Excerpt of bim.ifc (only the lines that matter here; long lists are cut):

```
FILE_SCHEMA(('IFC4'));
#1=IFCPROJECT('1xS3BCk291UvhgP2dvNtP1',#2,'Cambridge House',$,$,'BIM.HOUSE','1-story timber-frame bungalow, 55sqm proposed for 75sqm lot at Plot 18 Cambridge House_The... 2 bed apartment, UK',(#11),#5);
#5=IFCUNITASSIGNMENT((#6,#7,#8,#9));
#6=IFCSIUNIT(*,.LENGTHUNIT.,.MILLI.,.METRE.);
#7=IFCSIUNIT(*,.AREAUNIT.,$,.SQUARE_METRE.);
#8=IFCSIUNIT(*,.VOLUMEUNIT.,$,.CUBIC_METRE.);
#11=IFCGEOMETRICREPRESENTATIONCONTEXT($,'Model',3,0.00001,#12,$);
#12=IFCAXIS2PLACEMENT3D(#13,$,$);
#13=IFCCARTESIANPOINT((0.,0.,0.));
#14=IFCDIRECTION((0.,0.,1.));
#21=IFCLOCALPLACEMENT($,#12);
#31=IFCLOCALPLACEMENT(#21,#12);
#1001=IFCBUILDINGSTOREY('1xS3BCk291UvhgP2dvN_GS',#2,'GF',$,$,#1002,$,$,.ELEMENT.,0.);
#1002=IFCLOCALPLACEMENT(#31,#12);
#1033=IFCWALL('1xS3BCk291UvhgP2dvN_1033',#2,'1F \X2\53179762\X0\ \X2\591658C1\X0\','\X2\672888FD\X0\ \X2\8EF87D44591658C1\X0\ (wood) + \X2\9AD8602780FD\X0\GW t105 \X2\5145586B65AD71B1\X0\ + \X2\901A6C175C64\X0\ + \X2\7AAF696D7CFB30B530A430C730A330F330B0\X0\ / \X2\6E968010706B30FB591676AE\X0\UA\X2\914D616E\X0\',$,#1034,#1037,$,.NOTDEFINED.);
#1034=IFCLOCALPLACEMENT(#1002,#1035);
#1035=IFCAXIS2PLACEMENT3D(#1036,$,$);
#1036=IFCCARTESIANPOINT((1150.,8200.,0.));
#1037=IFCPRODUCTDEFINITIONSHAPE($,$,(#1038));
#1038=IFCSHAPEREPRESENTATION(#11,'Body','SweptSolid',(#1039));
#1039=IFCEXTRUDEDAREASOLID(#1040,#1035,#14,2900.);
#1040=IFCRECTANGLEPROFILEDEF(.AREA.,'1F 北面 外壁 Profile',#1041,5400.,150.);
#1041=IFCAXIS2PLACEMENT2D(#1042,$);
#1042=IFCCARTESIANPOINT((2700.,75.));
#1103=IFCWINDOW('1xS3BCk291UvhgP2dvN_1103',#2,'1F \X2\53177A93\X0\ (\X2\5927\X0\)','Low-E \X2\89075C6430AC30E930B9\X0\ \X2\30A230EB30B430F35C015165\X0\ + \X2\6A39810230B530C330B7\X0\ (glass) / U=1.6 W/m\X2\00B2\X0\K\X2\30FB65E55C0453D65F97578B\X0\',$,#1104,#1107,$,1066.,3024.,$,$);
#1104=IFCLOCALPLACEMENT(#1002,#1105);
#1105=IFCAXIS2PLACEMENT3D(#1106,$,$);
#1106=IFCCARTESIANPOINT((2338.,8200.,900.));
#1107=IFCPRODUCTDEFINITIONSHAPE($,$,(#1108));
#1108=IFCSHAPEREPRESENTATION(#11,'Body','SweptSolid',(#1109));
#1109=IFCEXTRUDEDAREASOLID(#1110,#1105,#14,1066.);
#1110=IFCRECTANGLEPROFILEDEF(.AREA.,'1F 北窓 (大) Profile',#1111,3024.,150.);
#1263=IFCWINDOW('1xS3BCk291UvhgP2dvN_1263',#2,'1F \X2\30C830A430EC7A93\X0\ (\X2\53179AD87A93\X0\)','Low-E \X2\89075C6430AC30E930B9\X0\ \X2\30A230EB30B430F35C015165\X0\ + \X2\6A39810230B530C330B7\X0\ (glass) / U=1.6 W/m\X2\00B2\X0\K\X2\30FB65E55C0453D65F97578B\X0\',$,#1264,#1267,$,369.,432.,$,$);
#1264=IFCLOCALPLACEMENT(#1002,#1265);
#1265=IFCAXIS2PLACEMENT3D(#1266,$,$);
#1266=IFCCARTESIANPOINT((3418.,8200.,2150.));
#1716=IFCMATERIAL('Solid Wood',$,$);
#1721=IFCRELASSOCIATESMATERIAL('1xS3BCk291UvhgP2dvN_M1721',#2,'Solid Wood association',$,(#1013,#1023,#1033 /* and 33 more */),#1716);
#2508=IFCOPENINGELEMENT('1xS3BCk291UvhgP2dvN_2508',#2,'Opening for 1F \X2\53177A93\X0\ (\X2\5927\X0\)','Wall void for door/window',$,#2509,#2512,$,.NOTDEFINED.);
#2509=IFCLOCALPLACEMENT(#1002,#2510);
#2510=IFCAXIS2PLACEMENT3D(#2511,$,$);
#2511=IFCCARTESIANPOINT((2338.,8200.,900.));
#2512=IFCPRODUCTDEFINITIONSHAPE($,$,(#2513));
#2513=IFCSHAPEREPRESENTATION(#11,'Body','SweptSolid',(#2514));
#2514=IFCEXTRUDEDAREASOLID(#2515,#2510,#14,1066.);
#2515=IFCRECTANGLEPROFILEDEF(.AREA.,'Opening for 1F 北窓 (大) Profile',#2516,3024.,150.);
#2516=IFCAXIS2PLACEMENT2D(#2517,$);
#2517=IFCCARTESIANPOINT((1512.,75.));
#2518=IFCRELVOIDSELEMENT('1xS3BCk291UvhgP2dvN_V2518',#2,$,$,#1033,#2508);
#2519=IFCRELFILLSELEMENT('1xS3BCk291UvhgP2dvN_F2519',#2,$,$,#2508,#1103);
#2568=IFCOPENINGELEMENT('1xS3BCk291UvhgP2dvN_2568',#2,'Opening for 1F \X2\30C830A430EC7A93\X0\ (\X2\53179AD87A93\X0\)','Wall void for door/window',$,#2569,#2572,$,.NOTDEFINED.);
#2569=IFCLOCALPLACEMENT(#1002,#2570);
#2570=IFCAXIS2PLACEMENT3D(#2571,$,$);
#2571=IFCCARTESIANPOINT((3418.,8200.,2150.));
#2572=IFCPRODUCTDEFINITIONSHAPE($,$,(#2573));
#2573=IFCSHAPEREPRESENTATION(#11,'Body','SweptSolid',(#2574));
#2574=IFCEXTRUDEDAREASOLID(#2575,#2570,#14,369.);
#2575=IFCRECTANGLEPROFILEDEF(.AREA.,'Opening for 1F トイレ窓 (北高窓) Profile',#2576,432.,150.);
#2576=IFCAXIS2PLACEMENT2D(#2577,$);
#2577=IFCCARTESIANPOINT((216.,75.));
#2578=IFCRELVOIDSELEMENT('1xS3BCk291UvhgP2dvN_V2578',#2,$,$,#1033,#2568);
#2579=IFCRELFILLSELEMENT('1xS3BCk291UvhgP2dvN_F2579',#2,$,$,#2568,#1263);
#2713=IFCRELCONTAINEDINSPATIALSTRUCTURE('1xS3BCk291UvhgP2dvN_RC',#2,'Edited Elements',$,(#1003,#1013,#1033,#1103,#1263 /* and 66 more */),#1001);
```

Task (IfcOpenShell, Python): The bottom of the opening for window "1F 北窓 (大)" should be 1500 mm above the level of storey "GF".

```python
import numpy as np
import ifcopenshell
import ifcopenshell.api.geometry
import ifcopenshell.geom
import ifcopenshell.util.element
import ifcopenshell.util.placement
import ifcopenshell.util.shape
import ifcopenshell.util.unit

model = ifcopenshell.open("bim.ifc")
unit_scale = ifcopenshell.util.unit.calculate_unit_scale(model)

window = model.by_guid("1xS3BCk291UvhgP2dvN_1103")
opening = window.FillsVoids[0].RelatingOpeningElement
storey = ifcopenshell.util.element.get_container(window, ifc_class="IfcBuildingStorey")
level = ifcopenshell.util.placement.get_local_placement(storey.ObjectPlacement)[2, 3]

# The opening's origin need not be at the sill, so measure its lowest point.
shape = ifcopenshell.geom.create_shape(ifcopenshell.geom.settings(), opening)
bottom = ifcopenshell.util.shape.get_shape_bottom_elevation(shape, shape.geometry) / unit_scale
dz = level + 1500.0 - bottom

shift = np.array([0.0, 0.0, dz])
# The window is not placed relative to its opening, so move both.
for product in (opening, window):
    matrix = ifcopenshell.util.placement.get_local_placement(product.ObjectPlacement)
    matrix[:3, 3] += shift
    ifcopenshell.api.geometry.edit_object_placement(model, product=product, matrix=matrix, is_si=False)

print(f"moved by {dz * unit_scale:+.3f} m")

model.write("bim_updated.ifc")
```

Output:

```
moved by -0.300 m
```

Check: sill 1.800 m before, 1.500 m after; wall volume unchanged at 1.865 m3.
